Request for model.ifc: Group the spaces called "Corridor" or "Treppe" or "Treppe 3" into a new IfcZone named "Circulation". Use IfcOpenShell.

First a look at what the model holds.

```python
import ifcopenshell

model = ifcopenshell.open("model.ifc")
print(model.schema)
seen = {}
for space in model.by_type("IfcSpace"):
    seen[space.LongName] = seen.get(space.LongName, 0) + 1
for name, count in sorted(seen.items(), key=str):
    print(count, "x", name)
print("zones:", [z.Name for z in model.by_type("IfcZone")][:20])
```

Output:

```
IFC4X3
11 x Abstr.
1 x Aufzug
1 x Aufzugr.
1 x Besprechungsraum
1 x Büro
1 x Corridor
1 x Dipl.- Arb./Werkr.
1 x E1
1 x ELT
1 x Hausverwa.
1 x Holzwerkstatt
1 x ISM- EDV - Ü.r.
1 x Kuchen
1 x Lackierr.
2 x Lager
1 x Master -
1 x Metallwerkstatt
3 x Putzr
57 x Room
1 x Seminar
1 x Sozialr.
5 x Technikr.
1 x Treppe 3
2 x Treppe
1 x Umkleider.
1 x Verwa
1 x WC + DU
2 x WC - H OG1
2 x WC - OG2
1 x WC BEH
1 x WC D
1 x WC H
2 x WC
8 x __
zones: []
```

```python
import ifcopenshell
import ifcopenshell.api.group
import ifcopenshell.api.root

model = ifcopenshell.open("model.ifc")

names = {"Corridor", "Treppe", "Treppe 3"}
spaces = [s for s in model.by_type("IfcSpace") if s.LongName in names]

zone = ifcopenshell.api.root.create_entity(model, ifc_class="IfcZone", name="Circulation")
ifcopenshell.api.group.assign_group(model, products=spaces, group=zone)
print(len(spaces), "spaces in", zone.Name)

model.write("model_updated.ifc")
```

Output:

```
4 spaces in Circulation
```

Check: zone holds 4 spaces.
